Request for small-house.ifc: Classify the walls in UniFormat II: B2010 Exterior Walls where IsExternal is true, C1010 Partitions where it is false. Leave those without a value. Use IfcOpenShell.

First a look at what the model holds.

```python
import ifcopenshell
import ifcopenshell.util.element

model = ifcopenshell.open("small-house.ifc")
print(model.schema)
print("classifications:", [c.Name for c in model.by_type("IfcClassification")])
values = [ifcopenshell.util.element.get_pset(e, "Pset_WallCommon", "IsExternal") for e in model.by_type("IfcWall")]
for value in (True, False, None):
    print("IsExternal", value, values.count(value))
```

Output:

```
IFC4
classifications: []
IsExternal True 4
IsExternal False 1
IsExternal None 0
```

```python
import ifcopenshell
import ifcopenshell.api.classification
import ifcopenshell.util.element

model = ifcopenshell.open("small-house.ifc")

system = ifcopenshell.api.classification.add_classification(model, classification="UniFormat II")

walls = model.by_type("IfcWall")
external = {e: ifcopenshell.util.element.get_pset(e, "Pset_WallCommon", "IsExternal") for e in walls}
for flag, code, name in ((True, "B2010", "Exterior Walls"), (False, "C1010", "Partitions")):
    products = [e for e in walls if external[e] is flag]
    ifcopenshell.api.classification.add_reference(
        model, products=products, classification=system, identification=code, name=name
    )
    print(code, len(products))

model.write("small-house_v2.ifc")
```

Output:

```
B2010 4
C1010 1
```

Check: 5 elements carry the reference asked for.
